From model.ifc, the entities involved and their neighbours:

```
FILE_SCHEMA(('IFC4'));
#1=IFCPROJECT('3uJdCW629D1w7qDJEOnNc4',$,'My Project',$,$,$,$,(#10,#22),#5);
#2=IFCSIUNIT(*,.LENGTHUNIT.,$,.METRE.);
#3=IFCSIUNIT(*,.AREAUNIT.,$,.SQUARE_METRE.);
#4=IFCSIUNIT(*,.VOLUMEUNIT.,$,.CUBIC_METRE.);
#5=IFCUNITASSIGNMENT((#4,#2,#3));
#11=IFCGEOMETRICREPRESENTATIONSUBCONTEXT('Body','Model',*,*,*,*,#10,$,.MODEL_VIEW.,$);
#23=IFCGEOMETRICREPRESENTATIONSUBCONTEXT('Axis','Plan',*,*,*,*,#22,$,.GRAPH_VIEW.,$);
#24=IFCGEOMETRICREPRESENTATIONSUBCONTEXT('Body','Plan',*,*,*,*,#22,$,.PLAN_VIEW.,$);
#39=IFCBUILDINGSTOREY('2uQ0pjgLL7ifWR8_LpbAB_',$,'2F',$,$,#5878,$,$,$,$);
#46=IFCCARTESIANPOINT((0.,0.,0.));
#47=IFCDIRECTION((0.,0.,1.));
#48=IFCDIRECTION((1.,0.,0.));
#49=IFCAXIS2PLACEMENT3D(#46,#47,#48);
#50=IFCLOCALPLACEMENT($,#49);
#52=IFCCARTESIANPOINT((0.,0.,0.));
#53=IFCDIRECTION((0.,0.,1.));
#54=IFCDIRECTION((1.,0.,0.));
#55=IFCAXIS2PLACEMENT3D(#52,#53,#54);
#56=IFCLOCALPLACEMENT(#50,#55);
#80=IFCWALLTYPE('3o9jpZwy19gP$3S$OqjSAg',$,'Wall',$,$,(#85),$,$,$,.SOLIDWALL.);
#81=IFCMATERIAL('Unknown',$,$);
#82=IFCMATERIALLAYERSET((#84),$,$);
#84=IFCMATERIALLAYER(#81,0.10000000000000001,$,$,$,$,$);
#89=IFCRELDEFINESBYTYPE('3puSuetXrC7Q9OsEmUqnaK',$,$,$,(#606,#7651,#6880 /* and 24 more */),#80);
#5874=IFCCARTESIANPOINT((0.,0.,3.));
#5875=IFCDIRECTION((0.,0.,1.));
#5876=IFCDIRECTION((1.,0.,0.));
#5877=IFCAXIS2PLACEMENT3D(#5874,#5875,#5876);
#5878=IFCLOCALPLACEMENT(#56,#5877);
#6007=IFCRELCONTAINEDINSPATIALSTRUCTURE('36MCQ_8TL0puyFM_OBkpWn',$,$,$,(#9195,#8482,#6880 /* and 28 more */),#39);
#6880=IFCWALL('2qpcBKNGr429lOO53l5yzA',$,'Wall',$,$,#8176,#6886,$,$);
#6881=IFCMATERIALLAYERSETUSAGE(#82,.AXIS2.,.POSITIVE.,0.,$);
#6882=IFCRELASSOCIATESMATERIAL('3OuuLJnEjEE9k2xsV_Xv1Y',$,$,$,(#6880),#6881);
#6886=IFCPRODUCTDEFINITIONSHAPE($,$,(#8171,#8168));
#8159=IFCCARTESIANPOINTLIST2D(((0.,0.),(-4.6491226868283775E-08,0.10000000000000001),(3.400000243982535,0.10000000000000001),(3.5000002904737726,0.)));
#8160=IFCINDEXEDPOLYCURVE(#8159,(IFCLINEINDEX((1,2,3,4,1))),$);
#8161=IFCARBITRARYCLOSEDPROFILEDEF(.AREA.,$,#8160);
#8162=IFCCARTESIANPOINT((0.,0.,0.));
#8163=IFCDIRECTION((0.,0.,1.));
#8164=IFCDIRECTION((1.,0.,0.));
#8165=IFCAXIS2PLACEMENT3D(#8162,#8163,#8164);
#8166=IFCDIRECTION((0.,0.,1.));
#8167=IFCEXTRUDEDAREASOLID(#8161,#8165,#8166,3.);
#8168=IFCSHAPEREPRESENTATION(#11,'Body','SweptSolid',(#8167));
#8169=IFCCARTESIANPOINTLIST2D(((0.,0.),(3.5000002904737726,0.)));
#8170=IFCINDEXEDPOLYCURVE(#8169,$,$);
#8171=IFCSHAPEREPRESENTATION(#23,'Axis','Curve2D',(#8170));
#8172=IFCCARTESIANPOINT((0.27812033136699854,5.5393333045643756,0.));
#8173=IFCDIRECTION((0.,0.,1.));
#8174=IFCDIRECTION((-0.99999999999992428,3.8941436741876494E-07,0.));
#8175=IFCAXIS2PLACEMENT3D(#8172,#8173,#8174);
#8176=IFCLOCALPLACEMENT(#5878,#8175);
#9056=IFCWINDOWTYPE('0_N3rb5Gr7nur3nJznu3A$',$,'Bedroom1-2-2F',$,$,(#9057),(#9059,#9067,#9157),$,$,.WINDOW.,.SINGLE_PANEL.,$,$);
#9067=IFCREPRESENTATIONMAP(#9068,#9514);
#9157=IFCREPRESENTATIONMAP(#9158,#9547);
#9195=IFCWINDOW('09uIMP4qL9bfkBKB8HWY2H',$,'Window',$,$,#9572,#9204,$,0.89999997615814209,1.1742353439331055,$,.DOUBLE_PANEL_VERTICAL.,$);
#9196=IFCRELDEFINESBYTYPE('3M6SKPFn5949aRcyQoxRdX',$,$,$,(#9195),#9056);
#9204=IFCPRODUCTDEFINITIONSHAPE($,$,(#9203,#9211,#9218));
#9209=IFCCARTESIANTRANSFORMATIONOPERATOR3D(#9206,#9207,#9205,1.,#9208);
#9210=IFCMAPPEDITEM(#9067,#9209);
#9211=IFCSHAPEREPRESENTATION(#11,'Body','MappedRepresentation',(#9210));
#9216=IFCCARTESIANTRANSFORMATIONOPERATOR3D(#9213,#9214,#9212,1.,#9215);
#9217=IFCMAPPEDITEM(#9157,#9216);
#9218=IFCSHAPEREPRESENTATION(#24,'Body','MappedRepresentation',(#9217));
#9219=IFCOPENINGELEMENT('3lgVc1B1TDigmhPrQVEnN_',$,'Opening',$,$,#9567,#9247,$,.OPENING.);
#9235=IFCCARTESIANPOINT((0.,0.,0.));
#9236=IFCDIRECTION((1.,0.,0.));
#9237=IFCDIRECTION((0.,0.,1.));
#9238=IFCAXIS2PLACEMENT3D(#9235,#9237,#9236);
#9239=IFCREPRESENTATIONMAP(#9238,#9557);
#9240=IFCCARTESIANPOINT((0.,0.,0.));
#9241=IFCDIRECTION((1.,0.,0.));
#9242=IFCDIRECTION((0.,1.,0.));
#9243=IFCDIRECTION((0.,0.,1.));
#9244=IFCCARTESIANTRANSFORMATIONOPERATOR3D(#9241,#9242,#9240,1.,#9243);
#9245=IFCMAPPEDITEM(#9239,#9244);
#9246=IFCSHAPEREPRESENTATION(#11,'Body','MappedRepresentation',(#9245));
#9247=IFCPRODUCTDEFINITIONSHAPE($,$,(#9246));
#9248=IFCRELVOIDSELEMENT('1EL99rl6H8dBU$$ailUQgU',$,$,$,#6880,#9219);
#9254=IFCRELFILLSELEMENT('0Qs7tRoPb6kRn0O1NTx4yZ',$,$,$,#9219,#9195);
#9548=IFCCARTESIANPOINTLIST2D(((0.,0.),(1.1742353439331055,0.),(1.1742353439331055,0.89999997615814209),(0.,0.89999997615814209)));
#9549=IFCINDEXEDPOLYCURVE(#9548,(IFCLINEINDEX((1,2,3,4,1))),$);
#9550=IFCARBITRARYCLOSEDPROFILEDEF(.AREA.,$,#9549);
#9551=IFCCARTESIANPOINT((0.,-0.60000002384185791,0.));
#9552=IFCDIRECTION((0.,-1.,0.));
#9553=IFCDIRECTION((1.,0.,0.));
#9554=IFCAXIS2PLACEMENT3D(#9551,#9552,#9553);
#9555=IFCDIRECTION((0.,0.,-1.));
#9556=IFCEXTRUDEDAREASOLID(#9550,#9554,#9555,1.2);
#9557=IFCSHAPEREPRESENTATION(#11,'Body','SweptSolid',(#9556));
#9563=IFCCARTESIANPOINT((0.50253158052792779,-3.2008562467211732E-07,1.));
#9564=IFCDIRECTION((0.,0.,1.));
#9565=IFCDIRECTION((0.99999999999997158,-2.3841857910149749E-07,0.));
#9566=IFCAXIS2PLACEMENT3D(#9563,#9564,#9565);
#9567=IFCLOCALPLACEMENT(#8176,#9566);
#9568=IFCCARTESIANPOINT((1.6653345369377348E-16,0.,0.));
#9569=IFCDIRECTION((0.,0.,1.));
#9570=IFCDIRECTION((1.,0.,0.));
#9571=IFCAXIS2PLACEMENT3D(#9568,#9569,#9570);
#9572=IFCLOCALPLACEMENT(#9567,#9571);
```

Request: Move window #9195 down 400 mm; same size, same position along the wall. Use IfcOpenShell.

```python
import numpy as np
import ifcopenshell
import ifcopenshell.api.geometry
import ifcopenshell.util.placement
import ifcopenshell.util.unit

model = ifcopenshell.open("model.ifc")
unit_scale = ifcopenshell.util.unit.calculate_unit_scale(model)

window = model.by_id(9195)
opening = window.FillsVoids[0].RelatingOpeningElement
dz = -0.4

shift = np.array([0.0, 0.0, dz])
# The window is placed relative to its opening, so it follows when the opening moves.
matrix = ifcopenshell.util.placement.get_local_placement(opening.ObjectPlacement)
matrix[:3, 3] += shift
ifcopenshell.api.geometry.edit_object_placement(
    model, product=opening, matrix=matrix, is_si=False, should_transform_children=True
)

print(f"moved by {dz * unit_scale:+.3f} m")

model.write("model_v2.ifc")
```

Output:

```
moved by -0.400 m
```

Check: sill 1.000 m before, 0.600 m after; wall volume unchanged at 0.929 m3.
